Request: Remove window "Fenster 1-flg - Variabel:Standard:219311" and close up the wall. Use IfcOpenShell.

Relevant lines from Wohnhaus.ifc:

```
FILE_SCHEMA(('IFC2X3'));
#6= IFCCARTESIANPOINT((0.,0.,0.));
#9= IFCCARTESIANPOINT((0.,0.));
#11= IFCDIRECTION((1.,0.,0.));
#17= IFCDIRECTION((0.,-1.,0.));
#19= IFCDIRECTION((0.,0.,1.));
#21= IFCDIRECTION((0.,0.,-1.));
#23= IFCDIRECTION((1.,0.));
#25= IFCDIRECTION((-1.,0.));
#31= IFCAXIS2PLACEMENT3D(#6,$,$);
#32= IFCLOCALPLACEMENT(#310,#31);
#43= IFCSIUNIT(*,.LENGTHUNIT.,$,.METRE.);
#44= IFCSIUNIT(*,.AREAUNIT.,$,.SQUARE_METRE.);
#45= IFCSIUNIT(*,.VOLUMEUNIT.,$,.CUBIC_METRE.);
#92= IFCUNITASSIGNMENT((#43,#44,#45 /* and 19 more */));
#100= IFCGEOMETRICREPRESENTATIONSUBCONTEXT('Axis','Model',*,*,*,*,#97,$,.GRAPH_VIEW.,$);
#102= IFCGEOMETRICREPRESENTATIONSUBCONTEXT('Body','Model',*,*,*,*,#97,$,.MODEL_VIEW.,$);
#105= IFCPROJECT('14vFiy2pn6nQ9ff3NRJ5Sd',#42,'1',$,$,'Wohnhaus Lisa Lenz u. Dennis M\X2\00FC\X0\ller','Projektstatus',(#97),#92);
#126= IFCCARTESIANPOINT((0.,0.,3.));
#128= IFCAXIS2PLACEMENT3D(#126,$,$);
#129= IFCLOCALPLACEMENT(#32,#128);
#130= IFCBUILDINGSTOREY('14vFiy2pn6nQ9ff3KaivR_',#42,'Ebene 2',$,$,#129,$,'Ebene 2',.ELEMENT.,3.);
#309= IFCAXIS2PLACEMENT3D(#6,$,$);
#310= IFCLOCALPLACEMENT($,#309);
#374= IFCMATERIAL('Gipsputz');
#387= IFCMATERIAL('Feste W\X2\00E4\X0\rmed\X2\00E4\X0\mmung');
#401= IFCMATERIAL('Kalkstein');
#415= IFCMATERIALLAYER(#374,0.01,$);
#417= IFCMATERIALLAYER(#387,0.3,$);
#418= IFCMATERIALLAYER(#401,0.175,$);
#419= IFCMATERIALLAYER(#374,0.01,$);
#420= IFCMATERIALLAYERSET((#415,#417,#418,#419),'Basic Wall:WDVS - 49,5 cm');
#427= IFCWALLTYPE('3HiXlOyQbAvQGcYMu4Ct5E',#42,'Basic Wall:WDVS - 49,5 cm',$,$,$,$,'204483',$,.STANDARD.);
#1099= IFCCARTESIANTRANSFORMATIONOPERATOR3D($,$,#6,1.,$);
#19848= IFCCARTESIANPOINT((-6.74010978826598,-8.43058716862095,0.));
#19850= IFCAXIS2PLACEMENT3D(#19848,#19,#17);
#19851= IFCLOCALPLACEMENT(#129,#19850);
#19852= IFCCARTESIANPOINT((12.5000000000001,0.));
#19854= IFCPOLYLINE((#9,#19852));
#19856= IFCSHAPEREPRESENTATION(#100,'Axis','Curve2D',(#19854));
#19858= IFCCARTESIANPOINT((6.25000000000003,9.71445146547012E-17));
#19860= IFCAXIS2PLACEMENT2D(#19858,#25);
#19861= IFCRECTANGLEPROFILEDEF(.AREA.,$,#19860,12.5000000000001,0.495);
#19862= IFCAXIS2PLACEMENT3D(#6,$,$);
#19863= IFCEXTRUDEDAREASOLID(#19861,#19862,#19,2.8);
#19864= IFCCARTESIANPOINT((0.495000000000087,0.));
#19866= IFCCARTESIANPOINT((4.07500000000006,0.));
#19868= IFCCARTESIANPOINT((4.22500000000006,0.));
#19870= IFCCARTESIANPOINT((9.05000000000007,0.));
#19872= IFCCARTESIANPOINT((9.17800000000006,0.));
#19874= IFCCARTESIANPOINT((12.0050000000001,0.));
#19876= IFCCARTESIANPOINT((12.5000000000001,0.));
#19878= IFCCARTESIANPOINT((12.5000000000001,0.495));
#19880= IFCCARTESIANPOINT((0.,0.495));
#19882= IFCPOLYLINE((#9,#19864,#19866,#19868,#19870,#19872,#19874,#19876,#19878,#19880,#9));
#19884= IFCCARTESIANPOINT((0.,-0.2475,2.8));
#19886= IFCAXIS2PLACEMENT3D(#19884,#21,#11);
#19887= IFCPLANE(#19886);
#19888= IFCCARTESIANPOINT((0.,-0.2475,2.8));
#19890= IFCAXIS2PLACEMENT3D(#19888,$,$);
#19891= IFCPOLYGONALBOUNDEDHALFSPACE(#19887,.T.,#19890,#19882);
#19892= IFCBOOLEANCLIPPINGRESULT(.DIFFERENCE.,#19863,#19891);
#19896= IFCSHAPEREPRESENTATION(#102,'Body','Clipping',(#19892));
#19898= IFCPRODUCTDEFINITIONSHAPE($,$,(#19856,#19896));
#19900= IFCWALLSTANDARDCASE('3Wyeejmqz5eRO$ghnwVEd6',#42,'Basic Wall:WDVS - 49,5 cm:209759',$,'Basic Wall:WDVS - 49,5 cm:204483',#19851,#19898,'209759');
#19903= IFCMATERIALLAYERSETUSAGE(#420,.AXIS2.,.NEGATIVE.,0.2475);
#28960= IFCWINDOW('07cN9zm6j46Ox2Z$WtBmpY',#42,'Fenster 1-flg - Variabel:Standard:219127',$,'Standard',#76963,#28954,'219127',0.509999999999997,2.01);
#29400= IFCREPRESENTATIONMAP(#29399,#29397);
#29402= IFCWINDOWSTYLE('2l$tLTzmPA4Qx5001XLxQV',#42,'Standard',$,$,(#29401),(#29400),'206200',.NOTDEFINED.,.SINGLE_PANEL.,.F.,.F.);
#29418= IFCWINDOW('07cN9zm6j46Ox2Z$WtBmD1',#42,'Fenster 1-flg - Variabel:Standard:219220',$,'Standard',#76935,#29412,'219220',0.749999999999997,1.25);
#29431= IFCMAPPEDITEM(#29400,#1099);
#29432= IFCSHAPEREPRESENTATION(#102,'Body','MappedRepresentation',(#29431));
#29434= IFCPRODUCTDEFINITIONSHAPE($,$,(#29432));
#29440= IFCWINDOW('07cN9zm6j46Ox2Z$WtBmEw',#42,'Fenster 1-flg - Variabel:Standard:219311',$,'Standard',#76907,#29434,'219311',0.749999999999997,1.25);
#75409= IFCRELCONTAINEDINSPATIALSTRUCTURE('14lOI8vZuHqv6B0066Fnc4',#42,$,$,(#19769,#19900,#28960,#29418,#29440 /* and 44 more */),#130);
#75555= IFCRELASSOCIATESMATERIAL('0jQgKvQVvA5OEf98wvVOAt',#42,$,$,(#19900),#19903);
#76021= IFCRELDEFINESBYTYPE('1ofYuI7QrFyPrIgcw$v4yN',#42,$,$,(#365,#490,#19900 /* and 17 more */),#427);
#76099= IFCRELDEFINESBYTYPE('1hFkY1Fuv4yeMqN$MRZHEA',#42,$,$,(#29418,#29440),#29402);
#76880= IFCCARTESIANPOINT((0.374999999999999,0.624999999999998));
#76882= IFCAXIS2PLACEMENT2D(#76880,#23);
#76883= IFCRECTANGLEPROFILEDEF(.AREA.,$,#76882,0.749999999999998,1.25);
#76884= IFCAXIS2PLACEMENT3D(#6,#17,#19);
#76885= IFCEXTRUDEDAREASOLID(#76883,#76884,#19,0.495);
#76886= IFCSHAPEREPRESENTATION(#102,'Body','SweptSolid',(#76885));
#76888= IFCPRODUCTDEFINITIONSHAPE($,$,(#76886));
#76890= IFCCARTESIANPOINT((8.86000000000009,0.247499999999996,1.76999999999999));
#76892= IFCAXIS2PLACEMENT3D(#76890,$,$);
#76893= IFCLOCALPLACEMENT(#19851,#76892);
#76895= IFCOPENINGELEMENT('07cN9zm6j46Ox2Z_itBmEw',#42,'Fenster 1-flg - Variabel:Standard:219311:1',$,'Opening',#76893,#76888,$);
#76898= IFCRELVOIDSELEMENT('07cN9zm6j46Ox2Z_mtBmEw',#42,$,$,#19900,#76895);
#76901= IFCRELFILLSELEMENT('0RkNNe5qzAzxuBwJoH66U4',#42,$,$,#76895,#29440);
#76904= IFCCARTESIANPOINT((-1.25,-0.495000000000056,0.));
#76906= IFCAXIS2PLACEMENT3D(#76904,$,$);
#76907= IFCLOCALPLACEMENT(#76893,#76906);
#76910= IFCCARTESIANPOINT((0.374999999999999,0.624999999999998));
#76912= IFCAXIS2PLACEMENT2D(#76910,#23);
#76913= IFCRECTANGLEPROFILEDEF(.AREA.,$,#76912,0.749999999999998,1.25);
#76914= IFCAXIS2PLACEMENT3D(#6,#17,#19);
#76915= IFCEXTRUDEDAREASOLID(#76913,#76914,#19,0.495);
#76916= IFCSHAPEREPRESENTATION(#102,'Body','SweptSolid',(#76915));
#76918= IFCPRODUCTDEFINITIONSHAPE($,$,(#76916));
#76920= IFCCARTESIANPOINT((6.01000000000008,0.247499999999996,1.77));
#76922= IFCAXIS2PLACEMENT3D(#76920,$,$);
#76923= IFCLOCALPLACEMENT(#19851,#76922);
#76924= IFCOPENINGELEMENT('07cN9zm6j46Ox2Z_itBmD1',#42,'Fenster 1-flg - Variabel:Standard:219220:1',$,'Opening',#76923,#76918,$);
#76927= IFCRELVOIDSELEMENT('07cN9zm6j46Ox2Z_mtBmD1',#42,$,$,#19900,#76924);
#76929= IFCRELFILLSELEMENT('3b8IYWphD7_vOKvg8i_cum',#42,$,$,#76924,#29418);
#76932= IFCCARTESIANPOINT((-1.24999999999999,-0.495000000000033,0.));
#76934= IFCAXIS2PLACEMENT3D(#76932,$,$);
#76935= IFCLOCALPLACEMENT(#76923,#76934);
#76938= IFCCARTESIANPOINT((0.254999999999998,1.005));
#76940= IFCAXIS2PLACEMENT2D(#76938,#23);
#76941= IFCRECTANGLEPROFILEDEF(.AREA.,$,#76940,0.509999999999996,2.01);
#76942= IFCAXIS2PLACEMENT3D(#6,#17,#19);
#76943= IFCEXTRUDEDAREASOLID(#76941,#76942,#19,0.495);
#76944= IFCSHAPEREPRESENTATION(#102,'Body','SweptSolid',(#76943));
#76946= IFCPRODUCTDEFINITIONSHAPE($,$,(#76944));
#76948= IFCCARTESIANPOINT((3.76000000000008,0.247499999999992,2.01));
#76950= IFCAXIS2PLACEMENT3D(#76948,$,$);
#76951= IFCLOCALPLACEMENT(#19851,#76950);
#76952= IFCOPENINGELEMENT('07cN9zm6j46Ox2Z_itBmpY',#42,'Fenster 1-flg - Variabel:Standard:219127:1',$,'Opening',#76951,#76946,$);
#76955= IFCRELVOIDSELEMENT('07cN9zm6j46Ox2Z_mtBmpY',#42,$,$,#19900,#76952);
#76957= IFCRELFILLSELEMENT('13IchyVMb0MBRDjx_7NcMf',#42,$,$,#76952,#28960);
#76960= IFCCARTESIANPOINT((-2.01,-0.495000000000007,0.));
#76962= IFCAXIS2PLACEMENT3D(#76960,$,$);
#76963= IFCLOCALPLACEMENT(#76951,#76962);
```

```python
import ifcopenshell
import ifcopenshell.api.feature
import ifcopenshell.api.root
import ifcopenshell.geom
import ifcopenshell.util.shape

model = ifcopenshell.open("Wohnhaus.ifc")
settings = ifcopenshell.geom.settings()


def volume(element):
    """Net volume in cubic metres, openings subtracted."""
    shape = ifcopenshell.geom.create_shape(settings, element)
    return ifcopenshell.util.shape.get_volume(shape.geometry)


window = model.by_guid("07cN9zm6j46Ox2Z$WtBmEw")
opening = window.FillsVoids[0].RelatingOpeningElement
wall = opening.VoidsElements[0].RelatingBuildingElement
before = volume(wall)

ifcopenshell.api.root.remove_product(model, product=window)
ifcopenshell.api.feature.remove_feature(model, feature=opening)

after = volume(wall)

print(f"wall volume {before:.3f} -> {after:.3f} m3")

model.write("Wohnhaus_rev.ifc")
```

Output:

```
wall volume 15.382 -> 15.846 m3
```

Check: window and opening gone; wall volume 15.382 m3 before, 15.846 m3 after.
